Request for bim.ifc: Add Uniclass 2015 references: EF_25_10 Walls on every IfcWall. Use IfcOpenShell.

First a look at what the model holds.

```python
import ifcopenshell

model = ifcopenshell.open("bim.ifc")
print(model.schema)
print("classifications:", [c.Name for c in model.by_type("IfcClassification")])
for ifc_class in ("IfcDoor", "IfcRoof", "IfcStair", "IfcWall", "IfcWindow"):
    print(ifc_class, len(model.by_type(ifc_class)))
```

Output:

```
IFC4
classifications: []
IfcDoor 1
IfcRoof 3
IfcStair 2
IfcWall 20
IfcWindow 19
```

```python
import ifcopenshell
import ifcopenshell.api.classification

model = ifcopenshell.open("bim.ifc")

system = ifcopenshell.api.classification.add_classification(model, classification="Uniclass 2015")

codes = {
    "IfcWall": ("EF_25_10", "Walls"),
}
for ifc_class, (code, name) in codes.items():
    products = model.by_type(ifc_class)
    ifcopenshell.api.classification.add_reference(
        model, products=products, classification=system, identification=code, name=name
    )
    print(code, len(products))

model.write("bim-out.ifc")
```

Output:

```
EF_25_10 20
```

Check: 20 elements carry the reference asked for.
